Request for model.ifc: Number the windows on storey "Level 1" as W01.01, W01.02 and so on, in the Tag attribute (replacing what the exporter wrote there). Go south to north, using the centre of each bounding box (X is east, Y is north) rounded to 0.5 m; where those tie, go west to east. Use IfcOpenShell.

First a look at what the model holds.

```python
import ifcopenshell
import ifcopenshell.util.element
import ifcopenshell.util.placement

model = ifcopenshell.open("model.ifc")
print(model.schema)
storey = next(s for s in model.by_type("IfcBuildingStorey") if s.Name == "Level 1")
windows = [e for e in ifcopenshell.util.element.get_decomposition(storey) if e.is_a("IfcWindow")]
for e in sorted(windows, key=lambda e: e.id()):
    origin = ifcopenshell.util.placement.get_local_placement(e.ObjectPlacement)[:3, 3]
    print(e.id(), e.Tag, e.Name, origin.round(2) + 0.0, sep=" | ")
```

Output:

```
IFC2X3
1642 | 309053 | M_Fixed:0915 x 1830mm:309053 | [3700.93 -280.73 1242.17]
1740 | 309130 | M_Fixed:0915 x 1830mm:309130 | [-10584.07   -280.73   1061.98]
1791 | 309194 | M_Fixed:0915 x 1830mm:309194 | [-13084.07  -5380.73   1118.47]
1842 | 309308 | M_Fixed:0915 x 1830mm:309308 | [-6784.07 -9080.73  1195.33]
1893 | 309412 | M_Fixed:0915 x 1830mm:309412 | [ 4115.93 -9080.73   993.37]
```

```python
import ifcopenshell
import ifcopenshell.geom
import ifcopenshell.util.element
import ifcopenshell.util.shape

model = ifcopenshell.open("model.ifc")
settings = ifcopenshell.geom.settings()
settings.set("use-world-coords", True)


def centre(element):
    shape = ifcopenshell.geom.create_shape(settings, element)
    return ifcopenshell.util.shape.get_bbox_centroid(shape.geometry)


storey = next(s for s in model.by_type("IfcBuildingStorey") if s.Name == "Level 1")
windows = [e for e in ifcopenshell.util.element.get_decomposition(storey) if e.is_a("IfcWindow")]

# Insertion points can sit at a corner or the storey origin, so sort by the geometry (in metres).
centres = {e: centre(e) for e in windows}
windows.sort(key=lambda e: (round(centres[e][1] / 0.5), centres[e][0]))

for i, e in enumerate(windows, start=1):
    number = f"W01.{i:02d}"
    e.Tag = number
    print(e.id(), number)

model.write("model_edited.ifc")
```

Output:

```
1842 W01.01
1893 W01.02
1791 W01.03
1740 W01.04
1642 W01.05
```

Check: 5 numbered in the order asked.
